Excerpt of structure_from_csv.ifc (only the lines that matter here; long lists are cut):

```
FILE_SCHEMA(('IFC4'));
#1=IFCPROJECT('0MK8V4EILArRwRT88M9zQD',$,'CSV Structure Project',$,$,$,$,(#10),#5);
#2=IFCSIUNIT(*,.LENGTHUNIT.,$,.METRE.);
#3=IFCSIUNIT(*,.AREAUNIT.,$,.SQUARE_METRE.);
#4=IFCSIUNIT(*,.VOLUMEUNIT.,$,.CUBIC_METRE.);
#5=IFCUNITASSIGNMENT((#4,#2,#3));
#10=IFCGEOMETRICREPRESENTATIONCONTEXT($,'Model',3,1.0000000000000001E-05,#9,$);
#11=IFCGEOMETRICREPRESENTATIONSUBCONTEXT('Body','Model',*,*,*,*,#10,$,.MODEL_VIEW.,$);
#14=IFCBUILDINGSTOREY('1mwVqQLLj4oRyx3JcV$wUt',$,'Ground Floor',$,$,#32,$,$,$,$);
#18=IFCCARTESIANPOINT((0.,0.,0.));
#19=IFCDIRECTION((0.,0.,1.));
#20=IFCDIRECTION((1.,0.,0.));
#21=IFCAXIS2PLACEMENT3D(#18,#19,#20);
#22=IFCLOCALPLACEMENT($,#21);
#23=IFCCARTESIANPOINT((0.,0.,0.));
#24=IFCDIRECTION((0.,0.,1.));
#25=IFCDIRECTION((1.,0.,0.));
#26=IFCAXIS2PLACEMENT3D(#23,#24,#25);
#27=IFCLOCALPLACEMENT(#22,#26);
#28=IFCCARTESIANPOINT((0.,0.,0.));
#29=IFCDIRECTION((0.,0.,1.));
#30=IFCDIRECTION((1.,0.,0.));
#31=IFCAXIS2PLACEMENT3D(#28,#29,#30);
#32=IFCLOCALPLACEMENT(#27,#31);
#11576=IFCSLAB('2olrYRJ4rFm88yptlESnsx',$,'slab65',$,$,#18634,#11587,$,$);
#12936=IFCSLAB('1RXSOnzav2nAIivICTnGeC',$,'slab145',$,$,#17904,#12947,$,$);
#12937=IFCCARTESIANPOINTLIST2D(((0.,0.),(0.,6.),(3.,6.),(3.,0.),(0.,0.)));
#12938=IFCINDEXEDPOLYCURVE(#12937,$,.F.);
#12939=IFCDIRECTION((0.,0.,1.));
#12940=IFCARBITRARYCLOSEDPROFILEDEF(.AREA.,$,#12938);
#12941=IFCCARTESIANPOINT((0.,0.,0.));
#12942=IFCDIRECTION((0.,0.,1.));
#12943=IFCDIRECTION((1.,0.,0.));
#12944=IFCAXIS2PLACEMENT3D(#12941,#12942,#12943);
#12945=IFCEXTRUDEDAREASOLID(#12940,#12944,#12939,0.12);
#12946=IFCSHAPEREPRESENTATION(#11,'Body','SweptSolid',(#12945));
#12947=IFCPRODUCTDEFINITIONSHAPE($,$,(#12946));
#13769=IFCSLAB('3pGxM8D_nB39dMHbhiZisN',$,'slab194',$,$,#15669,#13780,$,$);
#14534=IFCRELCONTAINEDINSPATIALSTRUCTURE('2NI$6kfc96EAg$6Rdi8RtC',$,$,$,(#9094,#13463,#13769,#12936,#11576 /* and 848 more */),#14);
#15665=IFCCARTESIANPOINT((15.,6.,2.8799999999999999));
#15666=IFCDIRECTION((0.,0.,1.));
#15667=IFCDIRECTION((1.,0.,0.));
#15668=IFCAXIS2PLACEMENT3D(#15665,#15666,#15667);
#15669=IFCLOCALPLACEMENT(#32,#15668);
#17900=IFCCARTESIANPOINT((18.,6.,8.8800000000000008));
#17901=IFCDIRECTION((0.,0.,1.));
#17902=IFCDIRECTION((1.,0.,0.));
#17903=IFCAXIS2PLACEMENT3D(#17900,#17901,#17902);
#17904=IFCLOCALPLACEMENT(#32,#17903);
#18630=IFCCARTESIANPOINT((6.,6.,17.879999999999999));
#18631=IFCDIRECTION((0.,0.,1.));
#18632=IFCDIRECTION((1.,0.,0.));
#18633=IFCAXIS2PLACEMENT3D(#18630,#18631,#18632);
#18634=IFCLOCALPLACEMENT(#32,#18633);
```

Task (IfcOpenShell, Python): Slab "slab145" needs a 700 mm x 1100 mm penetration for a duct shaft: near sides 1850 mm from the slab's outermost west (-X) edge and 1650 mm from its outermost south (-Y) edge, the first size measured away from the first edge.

```python
import numpy as np
import ifcopenshell
import ifcopenshell.api.feature
import ifcopenshell.api.geometry
import ifcopenshell.api.root
import ifcopenshell.geom
import ifcopenshell.util.placement
import ifcopenshell.util.representation
import ifcopenshell.util.shape
import ifcopenshell.util.unit

model = ifcopenshell.open("structure_from_csv.ifc")
unit_scale = ifcopenshell.util.unit.calculate_unit_scale(model)
settings = ifcopenshell.geom.settings()


def volume(element):
    """Net volume in cubic metres, openings subtracted."""
    shape = ifcopenshell.geom.create_shape(settings, element)
    return ifcopenshell.util.shape.get_volume(shape.geometry)


slab = model.by_id(12936)
before = volume(slab)

# Extent in the slab's own axes, in metres. The edges named are its -X and -Y sides.
slab_shape = ifcopenshell.geom.create_shape(settings, slab)
vertices = ifcopenshell.util.shape.get_vertices(slab_shape.geometry)
x_min, y_min, bottom = vertices.min(axis=0)
top = vertices[:, 2].max()

opening = ifcopenshell.api.root.create_entity(model, ifc_class="IfcOpeningElement", name="Duct shaft opening", predefined_type="OPENING")
context = ifcopenshell.util.representation.get_context(model, "Model", "Body", "MODEL_VIEW")
width, depth = 0.7, 1.1
outline = [(0.0, 0.0), (width, 0.0), (width, depth), (0.0, depth), (0.0, 0.0)]
# Overshoot both faces by 50 mm so the cut is clean.
shape = ifcopenshell.api.geometry.add_slab_representation(
    model, context=context, depth=top - bottom + 0.1, polyline=outline
)
ifcopenshell.api.geometry.assign_representation(model, product=opening, representation=shape)

matrix = ifcopenshell.util.placement.get_local_placement(slab.ObjectPlacement)
matrix[:, 3] = matrix @ np.append(np.array([x_min + 1.85, y_min + 1.65, bottom - 0.05]) / unit_scale, 1.0)
ifcopenshell.api.geometry.edit_object_placement(model, product=opening, matrix=matrix, is_si=False)
ifcopenshell.api.feature.add_feature(model, feature=opening, element=slab)

after = volume(slab)

print(f"slab volume {before:.3f} -> {after:.3f} m3")

model.write("structure_from_csv_v2.ifc")
```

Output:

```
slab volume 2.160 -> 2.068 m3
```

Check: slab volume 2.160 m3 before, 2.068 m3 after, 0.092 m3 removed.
